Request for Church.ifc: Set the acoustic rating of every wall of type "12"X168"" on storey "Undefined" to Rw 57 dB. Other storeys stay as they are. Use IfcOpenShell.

First a look at what the model holds.

```python
import ifcopenshell
import ifcopenshell.util.element

model = ifcopenshell.open("Church.ifc")
print(model.schema)
storey = next(s for s in model.by_type("IfcBuildingStorey") if s.Name == "Undefined")
walls = [e for e in ifcopenshell.util.element.get_decomposition(storey) if e.is_a("IfcWall")]
seen = {}
for e in walls:
    element_type = ifcopenshell.util.element.get_type(e)
    key = (element_type.Name if element_type != e and element_type else None, ifcopenshell.util.element.get_pset(e, "Pset_WallCommon", "AcousticRating"))
    seen[key] = seen.get(key, 0) + 1
for (name, value), count in sorted(seen.items(), key=str):
    print(count, "x", name, "|", value)
```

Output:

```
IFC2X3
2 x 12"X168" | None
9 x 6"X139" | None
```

```python
import ifcopenshell
import ifcopenshell.api.pset
import ifcopenshell.util.element

model = ifcopenshell.open("Church.ifc")

storey = next(s for s in model.by_type("IfcBuildingStorey") if s.Name == "Undefined")
walls = [e for e in ifcopenshell.util.element.get_decomposition(storey) if e.is_a("IfcWall")]

count = 0
for e in walls:
    element_type = ifcopenshell.util.element.get_type(e)
    if element_type in (None, e) or element_type.Name != '12"X168"':
        continue
    # add_pset returns the element's existing set when there is one.
    pset = ifcopenshell.api.pset.add_pset(model, product=e, name="Pset_WallCommon")
    ifcopenshell.api.pset.edit_pset(model, pset=pset, properties={"AcousticRating": "Rw 57 dB"})
    count += 1

print(count, "walls updated")

model.write("Church_edited.ifc")
```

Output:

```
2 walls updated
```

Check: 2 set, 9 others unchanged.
